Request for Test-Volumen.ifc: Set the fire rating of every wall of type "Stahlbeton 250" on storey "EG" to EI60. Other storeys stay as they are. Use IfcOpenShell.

First a look at what the model holds.

```python
import ifcopenshell
import ifcopenshell.util.element

model = ifcopenshell.open("Test-Volumen.ifc")
print(model.schema)
storey = next(s for s in model.by_type("IfcBuildingStorey") if s.Name == "EG")
walls = [e for e in ifcopenshell.util.element.get_decomposition(storey) if e.is_a("IfcWall")]
seen = {}
for e in walls:
    element_type = ifcopenshell.util.element.get_type(e)
    key = (element_type.Name if element_type != e and element_type else None, ifcopenshell.util.element.get_pset(e, "Pset_WallCommon", "FireRating"))
    seen[key] = seen.get(key, 0) + 1
for (name, value), count in sorted(seen.items(), key=str):
    print(count, "x", name, "|", value)
```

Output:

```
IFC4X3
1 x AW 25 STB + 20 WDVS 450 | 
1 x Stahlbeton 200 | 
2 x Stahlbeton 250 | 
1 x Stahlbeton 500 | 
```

```python
import ifcopenshell
import ifcopenshell.api.pset
import ifcopenshell.util.element

model = ifcopenshell.open("Test-Volumen.ifc")

storey = next(s for s in model.by_type("IfcBuildingStorey") if s.Name == "EG")
walls = [e for e in ifcopenshell.util.element.get_decomposition(storey) if e.is_a("IfcWall")]

count = 0
for e in walls:
    element_type = ifcopenshell.util.element.get_type(e)
    if element_type in (None, e) or element_type.Name != "Stahlbeton 250":
        continue
    # add_pset returns the element's existing set when there is one.
    pset = ifcopenshell.api.pset.add_pset(model, product=e, name="Pset_WallCommon")
    ifcopenshell.api.pset.edit_pset(model, pset=pset, properties={"FireRating": "EI60"})
    count += 1

print(count, "walls updated")

model.write("Test-Volumen-out.ifc")
```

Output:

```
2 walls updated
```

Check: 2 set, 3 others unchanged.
